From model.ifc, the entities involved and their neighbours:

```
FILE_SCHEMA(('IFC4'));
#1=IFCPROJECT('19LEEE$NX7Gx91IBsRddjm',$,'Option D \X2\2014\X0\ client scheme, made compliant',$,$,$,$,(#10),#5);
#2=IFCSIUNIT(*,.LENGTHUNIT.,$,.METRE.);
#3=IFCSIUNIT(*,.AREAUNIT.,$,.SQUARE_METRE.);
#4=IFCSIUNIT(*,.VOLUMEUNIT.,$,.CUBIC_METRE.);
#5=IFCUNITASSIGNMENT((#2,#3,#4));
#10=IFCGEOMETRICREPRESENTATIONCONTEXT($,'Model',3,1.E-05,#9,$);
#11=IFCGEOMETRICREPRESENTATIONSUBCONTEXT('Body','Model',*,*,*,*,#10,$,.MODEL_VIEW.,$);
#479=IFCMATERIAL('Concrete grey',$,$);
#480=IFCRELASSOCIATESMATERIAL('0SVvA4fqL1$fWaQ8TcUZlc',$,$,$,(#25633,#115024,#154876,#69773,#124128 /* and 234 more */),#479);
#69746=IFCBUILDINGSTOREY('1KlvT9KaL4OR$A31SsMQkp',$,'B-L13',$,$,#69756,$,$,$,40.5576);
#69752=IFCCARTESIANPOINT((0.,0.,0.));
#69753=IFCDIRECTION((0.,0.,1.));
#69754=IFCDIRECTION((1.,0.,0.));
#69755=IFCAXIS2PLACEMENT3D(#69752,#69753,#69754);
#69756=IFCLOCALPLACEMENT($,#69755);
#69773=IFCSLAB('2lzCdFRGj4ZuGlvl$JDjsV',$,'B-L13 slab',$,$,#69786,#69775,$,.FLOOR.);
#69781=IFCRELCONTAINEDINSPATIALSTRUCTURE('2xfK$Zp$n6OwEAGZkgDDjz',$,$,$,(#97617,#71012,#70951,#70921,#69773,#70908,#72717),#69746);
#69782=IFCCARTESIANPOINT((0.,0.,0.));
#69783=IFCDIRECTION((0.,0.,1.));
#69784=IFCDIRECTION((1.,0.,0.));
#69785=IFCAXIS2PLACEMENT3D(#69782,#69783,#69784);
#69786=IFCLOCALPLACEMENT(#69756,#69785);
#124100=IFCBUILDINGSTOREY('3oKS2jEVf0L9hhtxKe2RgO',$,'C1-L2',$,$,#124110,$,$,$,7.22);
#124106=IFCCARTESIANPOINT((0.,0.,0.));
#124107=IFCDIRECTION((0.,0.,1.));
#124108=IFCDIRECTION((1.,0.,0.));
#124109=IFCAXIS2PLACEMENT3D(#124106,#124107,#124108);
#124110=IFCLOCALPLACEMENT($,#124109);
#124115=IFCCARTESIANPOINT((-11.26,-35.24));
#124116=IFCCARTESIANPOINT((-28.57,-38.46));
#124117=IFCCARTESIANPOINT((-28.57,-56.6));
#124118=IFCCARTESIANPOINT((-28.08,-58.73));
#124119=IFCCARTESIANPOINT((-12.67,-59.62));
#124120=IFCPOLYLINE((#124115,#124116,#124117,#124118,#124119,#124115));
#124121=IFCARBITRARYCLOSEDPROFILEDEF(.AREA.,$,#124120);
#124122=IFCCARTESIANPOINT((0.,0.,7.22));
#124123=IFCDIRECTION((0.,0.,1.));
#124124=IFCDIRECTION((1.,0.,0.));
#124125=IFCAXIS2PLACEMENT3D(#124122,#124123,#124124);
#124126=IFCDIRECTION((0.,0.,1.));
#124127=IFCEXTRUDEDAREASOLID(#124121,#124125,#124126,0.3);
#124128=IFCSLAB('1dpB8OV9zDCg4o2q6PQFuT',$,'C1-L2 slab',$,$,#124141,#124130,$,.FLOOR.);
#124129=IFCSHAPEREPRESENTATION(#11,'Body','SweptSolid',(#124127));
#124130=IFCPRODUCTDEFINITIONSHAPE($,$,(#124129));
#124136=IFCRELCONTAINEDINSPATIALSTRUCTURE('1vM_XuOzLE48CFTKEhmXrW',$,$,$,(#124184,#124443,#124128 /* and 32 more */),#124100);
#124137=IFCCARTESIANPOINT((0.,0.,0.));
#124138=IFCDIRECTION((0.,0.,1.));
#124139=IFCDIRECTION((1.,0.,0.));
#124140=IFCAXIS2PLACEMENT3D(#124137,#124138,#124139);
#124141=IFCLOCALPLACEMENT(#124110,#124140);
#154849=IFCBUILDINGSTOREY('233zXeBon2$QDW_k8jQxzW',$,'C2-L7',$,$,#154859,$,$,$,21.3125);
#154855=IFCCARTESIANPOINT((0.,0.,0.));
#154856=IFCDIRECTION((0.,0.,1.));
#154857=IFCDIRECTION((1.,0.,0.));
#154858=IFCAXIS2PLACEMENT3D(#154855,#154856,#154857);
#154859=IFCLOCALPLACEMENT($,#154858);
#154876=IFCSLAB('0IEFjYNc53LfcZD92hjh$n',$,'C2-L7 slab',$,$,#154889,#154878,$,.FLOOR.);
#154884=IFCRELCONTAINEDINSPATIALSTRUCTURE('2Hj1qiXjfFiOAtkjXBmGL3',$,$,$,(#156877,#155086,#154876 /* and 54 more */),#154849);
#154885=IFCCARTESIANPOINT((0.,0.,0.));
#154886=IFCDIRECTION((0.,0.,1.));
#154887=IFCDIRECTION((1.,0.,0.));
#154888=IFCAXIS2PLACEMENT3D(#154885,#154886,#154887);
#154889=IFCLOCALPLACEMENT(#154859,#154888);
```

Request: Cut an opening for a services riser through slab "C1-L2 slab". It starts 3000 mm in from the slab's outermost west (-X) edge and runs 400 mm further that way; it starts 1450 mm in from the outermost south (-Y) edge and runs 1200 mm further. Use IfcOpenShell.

```python
import numpy as np
import ifcopenshell
import ifcopenshell.api.feature
import ifcopenshell.api.geometry
import ifcopenshell.api.root
import ifcopenshell.geom
import ifcopenshell.util.placement
import ifcopenshell.util.representation
import ifcopenshell.util.shape
import ifcopenshell.util.unit

model = ifcopenshell.open("model.ifc")
unit_scale = ifcopenshell.util.unit.calculate_unit_scale(model)
settings = ifcopenshell.geom.settings()


def volume(element):
    """Net volume in cubic metres, openings subtracted."""
    shape = ifcopenshell.geom.create_shape(settings, element)
    return ifcopenshell.util.shape.get_volume(shape.geometry)


slab = model.by_id(124128)
before = volume(slab)

# Extent in the slab's own axes, in metres. The edges named are its -X and -Y sides.
slab_shape = ifcopenshell.geom.create_shape(settings, slab)
vertices = ifcopenshell.util.shape.get_vertices(slab_shape.geometry)
x_min, y_min, bottom = vertices.min(axis=0)
top = vertices[:, 2].max()

opening = ifcopenshell.api.root.create_entity(model, ifc_class="IfcOpeningElement", name="Services riser opening", predefined_type="OPENING")
context = ifcopenshell.util.representation.get_context(model, "Model", "Body", "MODEL_VIEW")
width, depth = 0.4, 1.2
outline = [(0.0, 0.0), (width, 0.0), (width, depth), (0.0, depth), (0.0, 0.0)]
# Overshoot both faces by 50 mm so the cut is clean.
shape = ifcopenshell.api.geometry.add_slab_representation(
    model, context=context, depth=top - bottom + 0.1, polyline=outline
)
ifcopenshell.api.geometry.assign_representation(model, product=opening, representation=shape)

matrix = ifcopenshell.util.placement.get_local_placement(slab.ObjectPlacement)
matrix[:, 3] = matrix @ np.append(np.array([x_min + 3, y_min + 1.45, bottom - 0.05]) / unit_scale, 1.0)
ifcopenshell.api.geometry.edit_object_placement(model, product=opening, matrix=matrix, is_si=False)
ifcopenshell.api.feature.add_feature(model, feature=opening, element=slab)

after = volume(slab)

print(f"slab volume {before:.3f} -> {after:.3f} m3")

model.write("model_v2.ifc")
```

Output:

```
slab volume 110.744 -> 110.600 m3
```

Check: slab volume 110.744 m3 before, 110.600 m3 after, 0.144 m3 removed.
